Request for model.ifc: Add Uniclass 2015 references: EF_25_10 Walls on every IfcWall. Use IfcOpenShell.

First a look at what the model holds.

```python
import ifcopenshell

model = ifcopenshell.open("model.ifc")
print(model.schema)
print("classifications:", [c.Name for c in model.by_type("IfcClassification")])
for ifc_class in ("IfcDoor", "IfcRoof", "IfcStair", "IfcWall", "IfcWindow"):
    print(ifc_class, len(model.by_type(ifc_class)))
```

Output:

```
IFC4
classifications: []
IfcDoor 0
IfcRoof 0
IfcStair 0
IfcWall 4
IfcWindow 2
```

```python
import ifcopenshell
import ifcopenshell.api.classification

model = ifcopenshell.open("model.ifc")

system = ifcopenshell.api.classification.add_classification(model, classification="Uniclass 2015")

codes = {
    "IfcWall": ("EF_25_10", "Walls"),
}
for ifc_class, (code, name) in codes.items():
    products = model.by_type(ifc_class)
    ifcopenshell.api.classification.add_reference(
        model, products=products, classification=system, identification=code, name=name
    )
    print(code, len(products))

model.write("model_rev.ifc")
```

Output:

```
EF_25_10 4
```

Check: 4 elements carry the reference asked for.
